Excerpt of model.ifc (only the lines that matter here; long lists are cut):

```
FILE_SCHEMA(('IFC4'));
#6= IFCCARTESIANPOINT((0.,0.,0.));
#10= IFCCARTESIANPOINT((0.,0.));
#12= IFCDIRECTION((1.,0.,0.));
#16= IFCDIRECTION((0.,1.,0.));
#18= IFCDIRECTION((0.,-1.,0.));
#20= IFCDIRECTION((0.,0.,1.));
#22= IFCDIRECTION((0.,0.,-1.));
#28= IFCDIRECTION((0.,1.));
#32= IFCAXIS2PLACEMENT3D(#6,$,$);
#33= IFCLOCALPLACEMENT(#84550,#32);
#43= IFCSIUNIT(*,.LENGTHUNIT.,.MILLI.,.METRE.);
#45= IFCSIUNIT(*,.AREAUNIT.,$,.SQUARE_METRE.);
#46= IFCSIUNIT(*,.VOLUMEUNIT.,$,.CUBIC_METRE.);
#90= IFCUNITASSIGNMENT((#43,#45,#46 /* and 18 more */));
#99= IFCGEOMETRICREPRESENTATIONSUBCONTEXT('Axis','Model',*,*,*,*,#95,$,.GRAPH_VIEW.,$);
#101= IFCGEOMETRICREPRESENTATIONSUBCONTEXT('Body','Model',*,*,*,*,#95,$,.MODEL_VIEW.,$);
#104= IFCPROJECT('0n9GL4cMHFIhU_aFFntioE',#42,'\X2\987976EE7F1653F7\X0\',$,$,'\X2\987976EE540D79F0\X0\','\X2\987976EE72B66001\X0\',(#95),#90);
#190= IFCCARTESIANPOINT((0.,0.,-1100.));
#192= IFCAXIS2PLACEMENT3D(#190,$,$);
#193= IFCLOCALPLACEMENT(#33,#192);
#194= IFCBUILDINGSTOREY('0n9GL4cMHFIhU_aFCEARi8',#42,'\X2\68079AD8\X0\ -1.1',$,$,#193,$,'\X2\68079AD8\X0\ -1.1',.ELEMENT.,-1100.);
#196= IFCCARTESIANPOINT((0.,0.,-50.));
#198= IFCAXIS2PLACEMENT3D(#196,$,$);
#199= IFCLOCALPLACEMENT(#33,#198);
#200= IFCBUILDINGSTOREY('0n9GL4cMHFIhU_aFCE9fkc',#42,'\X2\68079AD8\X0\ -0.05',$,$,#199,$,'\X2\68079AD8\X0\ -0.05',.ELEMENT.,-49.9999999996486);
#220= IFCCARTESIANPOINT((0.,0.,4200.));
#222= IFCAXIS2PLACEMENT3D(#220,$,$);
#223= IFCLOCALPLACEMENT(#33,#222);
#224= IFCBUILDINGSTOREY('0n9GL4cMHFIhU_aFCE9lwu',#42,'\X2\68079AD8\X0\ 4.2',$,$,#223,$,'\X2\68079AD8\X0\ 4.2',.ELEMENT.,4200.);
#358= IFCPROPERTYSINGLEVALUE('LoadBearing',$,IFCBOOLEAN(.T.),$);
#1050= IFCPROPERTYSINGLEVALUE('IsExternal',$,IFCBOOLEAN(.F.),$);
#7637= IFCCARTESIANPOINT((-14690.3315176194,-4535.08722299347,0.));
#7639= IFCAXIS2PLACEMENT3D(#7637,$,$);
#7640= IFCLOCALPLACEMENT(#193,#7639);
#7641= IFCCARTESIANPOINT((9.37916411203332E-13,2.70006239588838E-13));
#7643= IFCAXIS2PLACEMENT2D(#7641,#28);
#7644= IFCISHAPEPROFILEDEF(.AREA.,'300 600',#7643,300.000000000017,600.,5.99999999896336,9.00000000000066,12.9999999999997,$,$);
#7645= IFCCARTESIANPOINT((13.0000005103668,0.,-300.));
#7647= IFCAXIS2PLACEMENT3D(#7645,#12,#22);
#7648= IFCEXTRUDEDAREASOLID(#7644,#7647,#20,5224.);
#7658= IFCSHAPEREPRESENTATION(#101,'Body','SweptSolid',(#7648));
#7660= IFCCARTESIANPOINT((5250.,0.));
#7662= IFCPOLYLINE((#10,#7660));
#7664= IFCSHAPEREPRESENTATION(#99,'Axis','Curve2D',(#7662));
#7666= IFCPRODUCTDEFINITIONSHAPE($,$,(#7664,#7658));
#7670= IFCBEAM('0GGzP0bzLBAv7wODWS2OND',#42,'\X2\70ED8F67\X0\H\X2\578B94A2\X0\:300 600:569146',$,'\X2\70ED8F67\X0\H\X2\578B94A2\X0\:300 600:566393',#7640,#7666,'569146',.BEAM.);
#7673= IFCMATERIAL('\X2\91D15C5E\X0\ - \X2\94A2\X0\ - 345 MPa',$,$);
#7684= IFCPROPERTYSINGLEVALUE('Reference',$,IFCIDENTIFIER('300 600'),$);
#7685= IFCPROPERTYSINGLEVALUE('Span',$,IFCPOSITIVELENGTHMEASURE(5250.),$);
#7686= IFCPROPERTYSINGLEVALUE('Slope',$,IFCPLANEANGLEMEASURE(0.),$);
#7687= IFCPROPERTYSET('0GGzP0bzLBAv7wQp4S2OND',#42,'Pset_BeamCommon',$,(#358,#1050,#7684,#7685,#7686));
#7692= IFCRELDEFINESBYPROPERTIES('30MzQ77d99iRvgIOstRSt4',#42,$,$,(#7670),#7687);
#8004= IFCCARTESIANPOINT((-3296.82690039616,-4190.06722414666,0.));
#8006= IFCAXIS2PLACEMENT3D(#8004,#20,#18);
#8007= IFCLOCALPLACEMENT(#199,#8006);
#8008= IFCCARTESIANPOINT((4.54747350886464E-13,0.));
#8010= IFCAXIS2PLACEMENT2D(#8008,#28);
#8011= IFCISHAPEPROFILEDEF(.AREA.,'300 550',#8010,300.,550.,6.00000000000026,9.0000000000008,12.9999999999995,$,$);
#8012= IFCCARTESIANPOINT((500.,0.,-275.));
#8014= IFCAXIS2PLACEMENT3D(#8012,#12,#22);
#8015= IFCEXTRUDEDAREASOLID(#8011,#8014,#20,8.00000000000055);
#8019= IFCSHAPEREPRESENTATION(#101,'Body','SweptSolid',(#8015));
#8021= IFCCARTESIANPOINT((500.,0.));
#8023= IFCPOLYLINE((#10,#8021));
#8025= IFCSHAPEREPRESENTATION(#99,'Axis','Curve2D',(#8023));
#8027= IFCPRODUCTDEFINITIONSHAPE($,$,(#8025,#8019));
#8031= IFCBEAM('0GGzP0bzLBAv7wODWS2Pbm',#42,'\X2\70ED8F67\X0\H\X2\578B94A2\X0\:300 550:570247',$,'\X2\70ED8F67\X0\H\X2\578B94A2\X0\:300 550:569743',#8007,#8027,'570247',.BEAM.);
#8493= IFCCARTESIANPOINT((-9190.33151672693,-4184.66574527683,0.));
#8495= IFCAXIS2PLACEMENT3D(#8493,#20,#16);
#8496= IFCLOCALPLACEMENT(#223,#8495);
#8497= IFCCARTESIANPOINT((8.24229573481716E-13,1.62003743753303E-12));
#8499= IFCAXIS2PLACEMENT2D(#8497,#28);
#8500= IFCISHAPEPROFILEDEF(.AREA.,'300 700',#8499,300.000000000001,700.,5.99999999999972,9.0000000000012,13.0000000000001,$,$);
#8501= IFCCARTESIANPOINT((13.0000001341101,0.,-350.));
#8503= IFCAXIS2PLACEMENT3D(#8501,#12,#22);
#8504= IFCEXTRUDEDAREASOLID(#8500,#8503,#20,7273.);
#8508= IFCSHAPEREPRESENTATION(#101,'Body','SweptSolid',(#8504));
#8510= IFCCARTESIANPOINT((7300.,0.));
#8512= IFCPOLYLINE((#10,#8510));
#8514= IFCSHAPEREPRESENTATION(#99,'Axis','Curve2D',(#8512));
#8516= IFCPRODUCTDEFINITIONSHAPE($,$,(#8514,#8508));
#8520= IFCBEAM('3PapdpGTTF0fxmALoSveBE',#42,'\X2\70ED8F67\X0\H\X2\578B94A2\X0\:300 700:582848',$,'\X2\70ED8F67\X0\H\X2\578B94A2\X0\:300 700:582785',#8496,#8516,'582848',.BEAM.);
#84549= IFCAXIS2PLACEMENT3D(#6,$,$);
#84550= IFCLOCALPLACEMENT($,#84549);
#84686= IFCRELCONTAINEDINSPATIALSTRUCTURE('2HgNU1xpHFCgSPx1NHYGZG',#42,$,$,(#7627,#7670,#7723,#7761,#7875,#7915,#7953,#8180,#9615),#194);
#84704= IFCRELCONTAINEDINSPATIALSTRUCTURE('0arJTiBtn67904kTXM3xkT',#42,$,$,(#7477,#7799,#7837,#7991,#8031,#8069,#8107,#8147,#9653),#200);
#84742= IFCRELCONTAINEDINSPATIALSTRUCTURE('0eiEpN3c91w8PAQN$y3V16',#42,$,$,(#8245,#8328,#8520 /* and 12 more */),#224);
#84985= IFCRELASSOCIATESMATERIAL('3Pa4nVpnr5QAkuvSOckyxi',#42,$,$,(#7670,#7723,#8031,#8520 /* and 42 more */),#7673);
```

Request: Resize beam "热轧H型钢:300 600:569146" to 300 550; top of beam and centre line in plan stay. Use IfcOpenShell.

```python
import ifcopenshell
import ifcopenshell.api.pset
import ifcopenshell.util.element
import ifcopenshell.util.representation

model = ifcopenshell.open("model.ifc")

member = model.by_guid("0GGzP0bzLBAv7wODWS2OND")
source = next(p for p in model.by_type("IfcIShapeProfileDef") if p.ProfileName == "300 550")

body = ifcopenshell.util.representation.get_representation(member, "Model", "Body")
solid = body.Items[0]
old_profile = solid.SweptArea

# Copy the section's sizes but keep this member's own profile position.
profile = ifcopenshell.util.element.copy(model, source)
# Profiles are centred, so shift by half the change in depth to hold the top.
shift = (old_profile.OverallDepth - profile.OverallDepth) / 2
x, y = old_profile.Position.Location.Coordinates
up = (-1.0, 0.0)  # upwards, in the solid's own plane
location = model.createIfcCartesianPoint((x + up[0] * shift, y + up[1] * shift))
profile.Position = model.createIfcAxis2Placement2D(location, old_profile.Position.RefDirection)
solid.SweptArea = profile
if not model.get_total_inverses(old_profile):
    ifcopenshell.util.element.remove_deep2(model, old_profile)
member.Name = member.Name.replace("300 600", "300 550")
member.ObjectType = member.ObjectType.replace("300 600", "300 550")
pset = model.by_id(ifcopenshell.util.element.get_pset(member, "Pset_BeamCommon", should_inherit=False)["id"])
ifcopenshell.api.pset.edit_pset(model, pset=pset, properties={"Reference": "300 550"})

print(solid.SweptArea)

model.write("model_v2.ifc")
```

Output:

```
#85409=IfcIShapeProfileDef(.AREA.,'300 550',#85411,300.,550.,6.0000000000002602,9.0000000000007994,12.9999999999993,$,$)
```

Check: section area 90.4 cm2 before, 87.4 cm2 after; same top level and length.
